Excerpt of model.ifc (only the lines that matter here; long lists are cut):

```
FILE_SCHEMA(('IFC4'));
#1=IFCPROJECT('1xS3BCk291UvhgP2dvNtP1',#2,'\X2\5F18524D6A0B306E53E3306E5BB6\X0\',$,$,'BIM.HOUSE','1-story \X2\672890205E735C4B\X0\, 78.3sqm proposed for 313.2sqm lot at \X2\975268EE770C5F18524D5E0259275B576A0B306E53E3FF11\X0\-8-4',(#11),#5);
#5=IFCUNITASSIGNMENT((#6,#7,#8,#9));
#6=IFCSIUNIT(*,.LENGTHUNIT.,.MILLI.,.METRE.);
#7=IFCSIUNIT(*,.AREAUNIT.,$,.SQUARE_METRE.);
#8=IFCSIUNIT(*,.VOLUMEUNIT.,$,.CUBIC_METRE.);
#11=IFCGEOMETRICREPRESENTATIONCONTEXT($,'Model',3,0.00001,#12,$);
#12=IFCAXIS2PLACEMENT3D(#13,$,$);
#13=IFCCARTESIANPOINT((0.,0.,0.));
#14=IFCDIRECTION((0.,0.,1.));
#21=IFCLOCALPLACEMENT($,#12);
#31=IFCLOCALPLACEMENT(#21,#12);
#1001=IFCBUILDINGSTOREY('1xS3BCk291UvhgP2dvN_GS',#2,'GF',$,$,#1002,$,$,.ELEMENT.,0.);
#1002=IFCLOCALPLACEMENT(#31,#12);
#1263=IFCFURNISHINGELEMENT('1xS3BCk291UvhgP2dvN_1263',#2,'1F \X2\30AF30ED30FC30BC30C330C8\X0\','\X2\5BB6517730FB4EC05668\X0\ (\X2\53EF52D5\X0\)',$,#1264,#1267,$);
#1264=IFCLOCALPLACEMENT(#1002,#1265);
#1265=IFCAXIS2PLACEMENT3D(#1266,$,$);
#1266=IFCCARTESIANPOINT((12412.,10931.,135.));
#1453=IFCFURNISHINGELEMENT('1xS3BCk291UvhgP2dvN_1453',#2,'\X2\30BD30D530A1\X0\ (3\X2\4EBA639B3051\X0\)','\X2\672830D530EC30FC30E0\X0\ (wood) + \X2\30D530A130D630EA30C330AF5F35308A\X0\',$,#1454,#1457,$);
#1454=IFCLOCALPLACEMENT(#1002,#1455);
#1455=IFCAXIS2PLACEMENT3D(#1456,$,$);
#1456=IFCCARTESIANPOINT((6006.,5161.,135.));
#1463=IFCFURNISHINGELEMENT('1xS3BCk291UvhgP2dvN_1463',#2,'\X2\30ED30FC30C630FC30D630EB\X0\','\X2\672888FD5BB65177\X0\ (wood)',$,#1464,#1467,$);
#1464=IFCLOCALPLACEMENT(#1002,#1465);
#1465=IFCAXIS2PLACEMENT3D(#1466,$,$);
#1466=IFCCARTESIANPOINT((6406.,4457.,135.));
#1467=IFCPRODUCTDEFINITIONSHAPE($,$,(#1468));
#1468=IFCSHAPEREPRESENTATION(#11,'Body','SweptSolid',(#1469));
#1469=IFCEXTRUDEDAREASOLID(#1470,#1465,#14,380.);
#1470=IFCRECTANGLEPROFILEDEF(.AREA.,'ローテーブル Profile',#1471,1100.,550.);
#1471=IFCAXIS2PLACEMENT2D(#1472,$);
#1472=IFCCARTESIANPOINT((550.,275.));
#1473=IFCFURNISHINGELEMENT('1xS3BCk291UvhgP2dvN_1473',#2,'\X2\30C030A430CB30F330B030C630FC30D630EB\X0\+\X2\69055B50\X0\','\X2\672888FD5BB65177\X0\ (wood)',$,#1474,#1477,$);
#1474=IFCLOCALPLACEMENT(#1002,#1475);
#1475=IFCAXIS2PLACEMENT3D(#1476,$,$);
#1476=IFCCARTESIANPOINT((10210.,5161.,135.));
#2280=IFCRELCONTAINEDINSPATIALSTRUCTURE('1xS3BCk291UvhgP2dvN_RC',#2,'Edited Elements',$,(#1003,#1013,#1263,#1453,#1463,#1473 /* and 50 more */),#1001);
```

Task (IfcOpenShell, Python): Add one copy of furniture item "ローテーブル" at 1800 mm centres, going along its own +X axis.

```python
import ifcopenshell
import ifcopenshell.api.geometry
import ifcopenshell.api.root
import ifcopenshell.util.element
import ifcopenshell.util.placement
import ifcopenshell.util.unit

model = ifcopenshell.open("model.ifc")
unit_scale = ifcopenshell.util.unit.calculate_unit_scale(model)


def reuse_history(source, copy):
    """copy_class also copies each property set's owner history, people and application; keep the originals."""
    for rel in copy.IsDefinedBy:
        if rel.is_a("IfcRelDefinesByProperties") and (history := rel.RelatingPropertyDefinition.OwnerHistory):
            rel.RelatingPropertyDefinition.OwnerHistory = source.OwnerHistory
            ifcopenshell.util.element.remove_deep2(model, history)


source = model.by_guid("1xS3BCk291UvhgP2dvN_1463")
base = ifcopenshell.util.placement.get_local_placement(source.ObjectPlacement)
step = base[:3, 0] * 1.8 / unit_scale

for i in range(1, 2):
    copy = ifcopenshell.api.root.copy_class(model, product=source)
    copy.Representation = ifcopenshell.util.element.copy_deep(
        model, source.Representation, exclude=["IfcGeometricRepresentationContext", "IfcRepresentationMap"]
    )
    reuse_history(source, copy)
    matrix = base.copy()
    matrix[:3, 3] += i * step
    print("added at", matrix[:3, 3].round(3) + 0.0)
    ifcopenshell.api.geometry.edit_object_placement(model, product=copy, matrix=matrix, is_si=False)

model.write("model_rev.ifc")
```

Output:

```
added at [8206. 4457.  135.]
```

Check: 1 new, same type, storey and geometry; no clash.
